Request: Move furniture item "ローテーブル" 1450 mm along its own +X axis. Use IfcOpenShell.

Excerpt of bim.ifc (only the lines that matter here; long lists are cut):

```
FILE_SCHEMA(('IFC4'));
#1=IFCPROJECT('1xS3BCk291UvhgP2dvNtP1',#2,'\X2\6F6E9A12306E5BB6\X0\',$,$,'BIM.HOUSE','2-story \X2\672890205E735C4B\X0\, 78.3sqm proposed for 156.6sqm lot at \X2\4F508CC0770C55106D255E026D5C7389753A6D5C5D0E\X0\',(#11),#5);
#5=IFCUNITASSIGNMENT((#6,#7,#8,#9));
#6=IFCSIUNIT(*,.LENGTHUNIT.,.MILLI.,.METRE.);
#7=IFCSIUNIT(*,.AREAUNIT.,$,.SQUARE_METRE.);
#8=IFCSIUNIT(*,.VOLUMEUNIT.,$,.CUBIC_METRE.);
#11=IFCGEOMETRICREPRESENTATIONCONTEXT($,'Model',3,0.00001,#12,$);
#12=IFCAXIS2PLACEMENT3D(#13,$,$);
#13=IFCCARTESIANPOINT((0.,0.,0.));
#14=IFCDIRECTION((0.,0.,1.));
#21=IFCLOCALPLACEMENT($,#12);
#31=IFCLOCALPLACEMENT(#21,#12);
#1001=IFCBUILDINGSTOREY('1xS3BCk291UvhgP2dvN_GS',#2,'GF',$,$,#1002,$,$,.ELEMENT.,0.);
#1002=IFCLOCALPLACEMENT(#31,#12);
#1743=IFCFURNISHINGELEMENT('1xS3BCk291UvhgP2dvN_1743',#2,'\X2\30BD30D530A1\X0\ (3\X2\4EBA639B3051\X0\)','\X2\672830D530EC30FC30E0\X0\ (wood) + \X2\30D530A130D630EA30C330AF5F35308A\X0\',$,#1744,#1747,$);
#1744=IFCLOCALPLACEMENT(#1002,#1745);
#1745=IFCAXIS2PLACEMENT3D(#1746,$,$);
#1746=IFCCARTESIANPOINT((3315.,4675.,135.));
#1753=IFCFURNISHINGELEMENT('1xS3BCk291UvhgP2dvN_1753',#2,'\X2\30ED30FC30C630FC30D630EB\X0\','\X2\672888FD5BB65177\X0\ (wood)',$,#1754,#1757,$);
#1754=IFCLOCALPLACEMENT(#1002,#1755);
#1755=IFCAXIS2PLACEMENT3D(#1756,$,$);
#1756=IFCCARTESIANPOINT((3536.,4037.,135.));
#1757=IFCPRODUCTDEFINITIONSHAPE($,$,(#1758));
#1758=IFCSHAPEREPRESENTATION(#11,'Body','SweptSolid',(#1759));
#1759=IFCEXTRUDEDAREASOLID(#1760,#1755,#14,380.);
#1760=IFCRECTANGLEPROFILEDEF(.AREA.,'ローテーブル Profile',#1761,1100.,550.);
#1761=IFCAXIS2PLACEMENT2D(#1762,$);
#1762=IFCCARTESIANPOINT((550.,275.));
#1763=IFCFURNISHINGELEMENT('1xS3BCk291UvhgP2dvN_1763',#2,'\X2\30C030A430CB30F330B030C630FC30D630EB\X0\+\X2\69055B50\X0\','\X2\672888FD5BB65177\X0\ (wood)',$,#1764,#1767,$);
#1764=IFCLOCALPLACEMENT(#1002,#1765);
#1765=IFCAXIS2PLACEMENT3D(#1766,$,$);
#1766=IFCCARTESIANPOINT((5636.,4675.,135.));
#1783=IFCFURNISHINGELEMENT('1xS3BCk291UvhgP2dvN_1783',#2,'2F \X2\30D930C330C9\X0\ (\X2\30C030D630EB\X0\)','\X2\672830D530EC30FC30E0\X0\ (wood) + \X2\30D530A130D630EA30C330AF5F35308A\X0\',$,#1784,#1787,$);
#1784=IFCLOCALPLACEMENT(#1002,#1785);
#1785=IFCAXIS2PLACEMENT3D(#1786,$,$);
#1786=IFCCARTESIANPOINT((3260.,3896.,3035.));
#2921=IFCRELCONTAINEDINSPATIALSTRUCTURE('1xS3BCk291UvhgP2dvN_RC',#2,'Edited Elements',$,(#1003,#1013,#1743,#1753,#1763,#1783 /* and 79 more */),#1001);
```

```python
import ifcopenshell
import ifcopenshell.api.geometry
import ifcopenshell.util.placement
import ifcopenshell.util.unit

model = ifcopenshell.open("bim.ifc")
unit_scale = ifcopenshell.util.unit.calculate_unit_scale(model)

item = model.by_guid("1xS3BCk291UvhgP2dvN_1753")
matrix = ifcopenshell.util.placement.get_local_placement(item.ObjectPlacement)
matrix[:3, 3] += matrix[:3, 0] * 1.45 / unit_scale
ifcopenshell.api.geometry.edit_object_placement(model, product=item, matrix=matrix, is_si=False)

print(ifcopenshell.util.placement.get_local_placement(item.ObjectPlacement).round(3) + 0.0)

model.write("bim-out.ifc")
```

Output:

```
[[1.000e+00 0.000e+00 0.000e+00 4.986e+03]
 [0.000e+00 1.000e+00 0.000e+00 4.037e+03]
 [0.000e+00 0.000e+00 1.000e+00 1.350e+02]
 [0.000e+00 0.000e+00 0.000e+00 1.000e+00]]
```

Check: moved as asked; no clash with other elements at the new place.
